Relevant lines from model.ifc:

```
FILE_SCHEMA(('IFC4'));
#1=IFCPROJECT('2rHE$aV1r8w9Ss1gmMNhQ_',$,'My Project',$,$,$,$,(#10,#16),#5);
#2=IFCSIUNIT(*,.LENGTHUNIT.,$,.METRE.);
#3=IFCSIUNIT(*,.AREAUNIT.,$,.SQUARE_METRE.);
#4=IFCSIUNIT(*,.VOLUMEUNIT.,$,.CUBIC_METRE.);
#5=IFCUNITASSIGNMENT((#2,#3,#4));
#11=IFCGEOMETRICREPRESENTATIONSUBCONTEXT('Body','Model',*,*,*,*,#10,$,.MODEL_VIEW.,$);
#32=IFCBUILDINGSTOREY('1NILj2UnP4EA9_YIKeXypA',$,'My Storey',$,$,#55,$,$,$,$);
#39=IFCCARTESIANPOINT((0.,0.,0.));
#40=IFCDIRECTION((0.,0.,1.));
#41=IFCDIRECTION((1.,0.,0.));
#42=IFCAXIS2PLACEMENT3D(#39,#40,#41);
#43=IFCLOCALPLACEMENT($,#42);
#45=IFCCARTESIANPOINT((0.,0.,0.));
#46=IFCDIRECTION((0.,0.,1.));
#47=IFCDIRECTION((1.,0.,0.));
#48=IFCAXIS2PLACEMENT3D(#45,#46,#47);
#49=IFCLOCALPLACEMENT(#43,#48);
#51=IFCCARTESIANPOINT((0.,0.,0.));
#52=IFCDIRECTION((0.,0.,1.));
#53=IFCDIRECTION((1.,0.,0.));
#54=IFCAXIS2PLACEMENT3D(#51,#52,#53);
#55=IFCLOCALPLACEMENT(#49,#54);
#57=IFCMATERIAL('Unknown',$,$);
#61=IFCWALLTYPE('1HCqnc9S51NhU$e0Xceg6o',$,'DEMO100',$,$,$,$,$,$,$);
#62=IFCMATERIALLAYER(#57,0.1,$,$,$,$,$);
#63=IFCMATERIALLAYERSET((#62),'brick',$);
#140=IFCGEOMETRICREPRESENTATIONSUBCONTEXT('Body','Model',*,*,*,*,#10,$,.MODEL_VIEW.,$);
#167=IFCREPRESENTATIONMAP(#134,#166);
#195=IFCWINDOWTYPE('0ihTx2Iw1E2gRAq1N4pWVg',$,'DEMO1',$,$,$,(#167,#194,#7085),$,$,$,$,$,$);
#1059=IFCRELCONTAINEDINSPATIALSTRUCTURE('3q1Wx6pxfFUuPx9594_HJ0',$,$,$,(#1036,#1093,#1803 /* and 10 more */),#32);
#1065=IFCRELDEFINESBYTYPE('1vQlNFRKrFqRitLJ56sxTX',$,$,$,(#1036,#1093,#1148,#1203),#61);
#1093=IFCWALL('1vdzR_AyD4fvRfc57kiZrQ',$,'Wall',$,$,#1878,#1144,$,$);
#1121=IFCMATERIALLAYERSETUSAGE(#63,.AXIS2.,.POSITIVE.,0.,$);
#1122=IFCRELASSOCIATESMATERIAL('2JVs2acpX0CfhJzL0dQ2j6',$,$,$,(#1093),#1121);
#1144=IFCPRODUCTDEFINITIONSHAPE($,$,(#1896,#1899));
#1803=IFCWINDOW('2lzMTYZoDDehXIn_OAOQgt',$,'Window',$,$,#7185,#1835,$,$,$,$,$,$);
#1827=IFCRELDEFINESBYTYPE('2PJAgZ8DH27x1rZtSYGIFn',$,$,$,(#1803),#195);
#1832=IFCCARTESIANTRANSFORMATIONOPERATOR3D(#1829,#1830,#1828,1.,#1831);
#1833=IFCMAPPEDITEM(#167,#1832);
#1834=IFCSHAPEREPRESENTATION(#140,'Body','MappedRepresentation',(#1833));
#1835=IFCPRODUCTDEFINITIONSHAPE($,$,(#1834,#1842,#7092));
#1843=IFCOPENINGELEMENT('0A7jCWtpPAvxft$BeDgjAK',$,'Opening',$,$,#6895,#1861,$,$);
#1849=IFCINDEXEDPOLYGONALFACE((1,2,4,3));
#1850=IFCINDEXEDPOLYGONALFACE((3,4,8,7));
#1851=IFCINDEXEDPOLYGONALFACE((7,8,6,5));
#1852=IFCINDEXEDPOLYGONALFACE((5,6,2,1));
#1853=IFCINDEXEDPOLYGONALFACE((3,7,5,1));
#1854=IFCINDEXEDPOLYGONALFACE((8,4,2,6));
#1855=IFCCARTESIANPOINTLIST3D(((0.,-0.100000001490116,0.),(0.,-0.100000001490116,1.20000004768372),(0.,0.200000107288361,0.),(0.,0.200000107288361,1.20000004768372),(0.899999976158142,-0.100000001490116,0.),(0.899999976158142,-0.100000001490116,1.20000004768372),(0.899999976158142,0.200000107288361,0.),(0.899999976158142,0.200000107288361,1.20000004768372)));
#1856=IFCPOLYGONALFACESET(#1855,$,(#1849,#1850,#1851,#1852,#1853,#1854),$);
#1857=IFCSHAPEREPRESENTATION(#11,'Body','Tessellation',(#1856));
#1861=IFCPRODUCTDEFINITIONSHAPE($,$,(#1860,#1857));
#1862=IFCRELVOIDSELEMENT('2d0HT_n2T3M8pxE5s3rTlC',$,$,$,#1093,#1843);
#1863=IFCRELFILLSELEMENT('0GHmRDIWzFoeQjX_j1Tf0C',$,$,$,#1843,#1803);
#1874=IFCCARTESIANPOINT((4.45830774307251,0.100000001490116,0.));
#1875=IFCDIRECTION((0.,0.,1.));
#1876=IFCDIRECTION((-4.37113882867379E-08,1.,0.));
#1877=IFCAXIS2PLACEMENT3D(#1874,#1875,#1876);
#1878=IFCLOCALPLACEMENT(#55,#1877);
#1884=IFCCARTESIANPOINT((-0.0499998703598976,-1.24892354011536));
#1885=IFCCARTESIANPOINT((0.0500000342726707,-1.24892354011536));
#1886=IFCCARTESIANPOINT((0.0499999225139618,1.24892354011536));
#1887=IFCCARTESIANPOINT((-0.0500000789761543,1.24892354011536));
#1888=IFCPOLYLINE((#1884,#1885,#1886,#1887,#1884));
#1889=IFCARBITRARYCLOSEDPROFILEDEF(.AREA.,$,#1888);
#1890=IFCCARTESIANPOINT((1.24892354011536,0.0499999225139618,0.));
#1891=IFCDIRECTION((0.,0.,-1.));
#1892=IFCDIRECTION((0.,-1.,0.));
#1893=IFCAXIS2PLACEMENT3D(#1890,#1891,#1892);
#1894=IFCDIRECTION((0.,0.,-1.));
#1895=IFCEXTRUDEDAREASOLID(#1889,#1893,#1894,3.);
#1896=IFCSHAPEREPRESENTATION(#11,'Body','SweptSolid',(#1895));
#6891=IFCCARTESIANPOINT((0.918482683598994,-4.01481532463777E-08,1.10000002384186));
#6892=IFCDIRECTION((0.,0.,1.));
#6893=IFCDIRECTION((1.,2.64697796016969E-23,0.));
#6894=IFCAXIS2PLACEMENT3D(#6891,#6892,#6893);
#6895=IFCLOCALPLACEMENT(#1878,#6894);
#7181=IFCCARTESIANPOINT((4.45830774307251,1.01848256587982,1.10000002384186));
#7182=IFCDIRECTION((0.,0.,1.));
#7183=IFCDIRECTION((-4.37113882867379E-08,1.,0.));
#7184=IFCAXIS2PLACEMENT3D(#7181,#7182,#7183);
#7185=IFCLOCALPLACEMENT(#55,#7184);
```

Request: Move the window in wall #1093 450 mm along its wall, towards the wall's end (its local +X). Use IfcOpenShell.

```python
import ifcopenshell
import ifcopenshell.api.geometry
import ifcopenshell.util.placement
import ifcopenshell.util.unit

model = ifcopenshell.open("model.ifc")
unit_scale = ifcopenshell.util.unit.calculate_unit_scale(model)

window = model.by_id(1803)
opening = window.FillsVoids[0].RelatingOpeningElement
wall = opening.VoidsElements[0].RelatingBuildingElement

wall_matrix = ifcopenshell.util.placement.get_local_placement(wall.ObjectPlacement)
shift = wall_matrix[:3, 0] * 0.45 / unit_scale
before = ifcopenshell.util.placement.get_local_placement(window.ObjectPlacement)[:3, 3].copy()

# The window is not placed relative to its opening, so move both.
for product in (opening, window):
    matrix = ifcopenshell.util.placement.get_local_placement(product.ObjectPlacement)
    matrix[:3, 3] += shift
    ifcopenshell.api.geometry.edit_object_placement(model, product=product, matrix=matrix, is_si=False)

after = ifcopenshell.util.placement.get_local_placement(window.ObjectPlacement)[:3, 3]
print("window moved by", (after - before).round(3) + 0.0)

model.write("model_updated.ifc")
```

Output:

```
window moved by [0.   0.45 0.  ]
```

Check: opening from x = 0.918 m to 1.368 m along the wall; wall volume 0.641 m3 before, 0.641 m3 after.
